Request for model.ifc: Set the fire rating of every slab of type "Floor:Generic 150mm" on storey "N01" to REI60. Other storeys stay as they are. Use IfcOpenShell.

First a look at what the model holds.

```python
import ifcopenshell
import ifcopenshell.util.element

model = ifcopenshell.open("model.ifc")
print(model.schema)
storey = next(s for s in model.by_type("IfcBuildingStorey") if s.Name == "N01")
slabs = [e for e in ifcopenshell.util.element.get_decomposition(storey) if e.is_a("IfcSlab")]
seen = {}
for e in slabs:
    element_type = ifcopenshell.util.element.get_type(e)
    key = (element_type.Name if element_type != e and element_type else None, ifcopenshell.util.element.get_pset(e, "Pset_SlabCommon", "FireRating"))
    seen[key] = seen.get(key, 0) + 1
for (name, value), count in sorted(seen.items(), key=str):
    print(count, "x", name, "|", value)
```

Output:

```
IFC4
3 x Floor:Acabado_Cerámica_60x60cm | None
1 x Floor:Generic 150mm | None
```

```python
import ifcopenshell
import ifcopenshell.api.pset
import ifcopenshell.util.element

model = ifcopenshell.open("model.ifc")

storey = next(s for s in model.by_type("IfcBuildingStorey") if s.Name == "N01")
slabs = [e for e in ifcopenshell.util.element.get_decomposition(storey) if e.is_a("IfcSlab")]

count = 0
for e in slabs:
    element_type = ifcopenshell.util.element.get_type(e)
    if element_type in (None, e) or element_type.Name != "Floor:Generic 150mm":
        continue
    # add_pset returns the element's existing set when there is one.
    pset = ifcopenshell.api.pset.add_pset(model, product=e, name="Pset_SlabCommon")
    ifcopenshell.api.pset.edit_pset(model, pset=pset, properties={"FireRating": "REI60"})
    count += 1

print(count, "slabs updated")

model.write("model_updated.ifc")
```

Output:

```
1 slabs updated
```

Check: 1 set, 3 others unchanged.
